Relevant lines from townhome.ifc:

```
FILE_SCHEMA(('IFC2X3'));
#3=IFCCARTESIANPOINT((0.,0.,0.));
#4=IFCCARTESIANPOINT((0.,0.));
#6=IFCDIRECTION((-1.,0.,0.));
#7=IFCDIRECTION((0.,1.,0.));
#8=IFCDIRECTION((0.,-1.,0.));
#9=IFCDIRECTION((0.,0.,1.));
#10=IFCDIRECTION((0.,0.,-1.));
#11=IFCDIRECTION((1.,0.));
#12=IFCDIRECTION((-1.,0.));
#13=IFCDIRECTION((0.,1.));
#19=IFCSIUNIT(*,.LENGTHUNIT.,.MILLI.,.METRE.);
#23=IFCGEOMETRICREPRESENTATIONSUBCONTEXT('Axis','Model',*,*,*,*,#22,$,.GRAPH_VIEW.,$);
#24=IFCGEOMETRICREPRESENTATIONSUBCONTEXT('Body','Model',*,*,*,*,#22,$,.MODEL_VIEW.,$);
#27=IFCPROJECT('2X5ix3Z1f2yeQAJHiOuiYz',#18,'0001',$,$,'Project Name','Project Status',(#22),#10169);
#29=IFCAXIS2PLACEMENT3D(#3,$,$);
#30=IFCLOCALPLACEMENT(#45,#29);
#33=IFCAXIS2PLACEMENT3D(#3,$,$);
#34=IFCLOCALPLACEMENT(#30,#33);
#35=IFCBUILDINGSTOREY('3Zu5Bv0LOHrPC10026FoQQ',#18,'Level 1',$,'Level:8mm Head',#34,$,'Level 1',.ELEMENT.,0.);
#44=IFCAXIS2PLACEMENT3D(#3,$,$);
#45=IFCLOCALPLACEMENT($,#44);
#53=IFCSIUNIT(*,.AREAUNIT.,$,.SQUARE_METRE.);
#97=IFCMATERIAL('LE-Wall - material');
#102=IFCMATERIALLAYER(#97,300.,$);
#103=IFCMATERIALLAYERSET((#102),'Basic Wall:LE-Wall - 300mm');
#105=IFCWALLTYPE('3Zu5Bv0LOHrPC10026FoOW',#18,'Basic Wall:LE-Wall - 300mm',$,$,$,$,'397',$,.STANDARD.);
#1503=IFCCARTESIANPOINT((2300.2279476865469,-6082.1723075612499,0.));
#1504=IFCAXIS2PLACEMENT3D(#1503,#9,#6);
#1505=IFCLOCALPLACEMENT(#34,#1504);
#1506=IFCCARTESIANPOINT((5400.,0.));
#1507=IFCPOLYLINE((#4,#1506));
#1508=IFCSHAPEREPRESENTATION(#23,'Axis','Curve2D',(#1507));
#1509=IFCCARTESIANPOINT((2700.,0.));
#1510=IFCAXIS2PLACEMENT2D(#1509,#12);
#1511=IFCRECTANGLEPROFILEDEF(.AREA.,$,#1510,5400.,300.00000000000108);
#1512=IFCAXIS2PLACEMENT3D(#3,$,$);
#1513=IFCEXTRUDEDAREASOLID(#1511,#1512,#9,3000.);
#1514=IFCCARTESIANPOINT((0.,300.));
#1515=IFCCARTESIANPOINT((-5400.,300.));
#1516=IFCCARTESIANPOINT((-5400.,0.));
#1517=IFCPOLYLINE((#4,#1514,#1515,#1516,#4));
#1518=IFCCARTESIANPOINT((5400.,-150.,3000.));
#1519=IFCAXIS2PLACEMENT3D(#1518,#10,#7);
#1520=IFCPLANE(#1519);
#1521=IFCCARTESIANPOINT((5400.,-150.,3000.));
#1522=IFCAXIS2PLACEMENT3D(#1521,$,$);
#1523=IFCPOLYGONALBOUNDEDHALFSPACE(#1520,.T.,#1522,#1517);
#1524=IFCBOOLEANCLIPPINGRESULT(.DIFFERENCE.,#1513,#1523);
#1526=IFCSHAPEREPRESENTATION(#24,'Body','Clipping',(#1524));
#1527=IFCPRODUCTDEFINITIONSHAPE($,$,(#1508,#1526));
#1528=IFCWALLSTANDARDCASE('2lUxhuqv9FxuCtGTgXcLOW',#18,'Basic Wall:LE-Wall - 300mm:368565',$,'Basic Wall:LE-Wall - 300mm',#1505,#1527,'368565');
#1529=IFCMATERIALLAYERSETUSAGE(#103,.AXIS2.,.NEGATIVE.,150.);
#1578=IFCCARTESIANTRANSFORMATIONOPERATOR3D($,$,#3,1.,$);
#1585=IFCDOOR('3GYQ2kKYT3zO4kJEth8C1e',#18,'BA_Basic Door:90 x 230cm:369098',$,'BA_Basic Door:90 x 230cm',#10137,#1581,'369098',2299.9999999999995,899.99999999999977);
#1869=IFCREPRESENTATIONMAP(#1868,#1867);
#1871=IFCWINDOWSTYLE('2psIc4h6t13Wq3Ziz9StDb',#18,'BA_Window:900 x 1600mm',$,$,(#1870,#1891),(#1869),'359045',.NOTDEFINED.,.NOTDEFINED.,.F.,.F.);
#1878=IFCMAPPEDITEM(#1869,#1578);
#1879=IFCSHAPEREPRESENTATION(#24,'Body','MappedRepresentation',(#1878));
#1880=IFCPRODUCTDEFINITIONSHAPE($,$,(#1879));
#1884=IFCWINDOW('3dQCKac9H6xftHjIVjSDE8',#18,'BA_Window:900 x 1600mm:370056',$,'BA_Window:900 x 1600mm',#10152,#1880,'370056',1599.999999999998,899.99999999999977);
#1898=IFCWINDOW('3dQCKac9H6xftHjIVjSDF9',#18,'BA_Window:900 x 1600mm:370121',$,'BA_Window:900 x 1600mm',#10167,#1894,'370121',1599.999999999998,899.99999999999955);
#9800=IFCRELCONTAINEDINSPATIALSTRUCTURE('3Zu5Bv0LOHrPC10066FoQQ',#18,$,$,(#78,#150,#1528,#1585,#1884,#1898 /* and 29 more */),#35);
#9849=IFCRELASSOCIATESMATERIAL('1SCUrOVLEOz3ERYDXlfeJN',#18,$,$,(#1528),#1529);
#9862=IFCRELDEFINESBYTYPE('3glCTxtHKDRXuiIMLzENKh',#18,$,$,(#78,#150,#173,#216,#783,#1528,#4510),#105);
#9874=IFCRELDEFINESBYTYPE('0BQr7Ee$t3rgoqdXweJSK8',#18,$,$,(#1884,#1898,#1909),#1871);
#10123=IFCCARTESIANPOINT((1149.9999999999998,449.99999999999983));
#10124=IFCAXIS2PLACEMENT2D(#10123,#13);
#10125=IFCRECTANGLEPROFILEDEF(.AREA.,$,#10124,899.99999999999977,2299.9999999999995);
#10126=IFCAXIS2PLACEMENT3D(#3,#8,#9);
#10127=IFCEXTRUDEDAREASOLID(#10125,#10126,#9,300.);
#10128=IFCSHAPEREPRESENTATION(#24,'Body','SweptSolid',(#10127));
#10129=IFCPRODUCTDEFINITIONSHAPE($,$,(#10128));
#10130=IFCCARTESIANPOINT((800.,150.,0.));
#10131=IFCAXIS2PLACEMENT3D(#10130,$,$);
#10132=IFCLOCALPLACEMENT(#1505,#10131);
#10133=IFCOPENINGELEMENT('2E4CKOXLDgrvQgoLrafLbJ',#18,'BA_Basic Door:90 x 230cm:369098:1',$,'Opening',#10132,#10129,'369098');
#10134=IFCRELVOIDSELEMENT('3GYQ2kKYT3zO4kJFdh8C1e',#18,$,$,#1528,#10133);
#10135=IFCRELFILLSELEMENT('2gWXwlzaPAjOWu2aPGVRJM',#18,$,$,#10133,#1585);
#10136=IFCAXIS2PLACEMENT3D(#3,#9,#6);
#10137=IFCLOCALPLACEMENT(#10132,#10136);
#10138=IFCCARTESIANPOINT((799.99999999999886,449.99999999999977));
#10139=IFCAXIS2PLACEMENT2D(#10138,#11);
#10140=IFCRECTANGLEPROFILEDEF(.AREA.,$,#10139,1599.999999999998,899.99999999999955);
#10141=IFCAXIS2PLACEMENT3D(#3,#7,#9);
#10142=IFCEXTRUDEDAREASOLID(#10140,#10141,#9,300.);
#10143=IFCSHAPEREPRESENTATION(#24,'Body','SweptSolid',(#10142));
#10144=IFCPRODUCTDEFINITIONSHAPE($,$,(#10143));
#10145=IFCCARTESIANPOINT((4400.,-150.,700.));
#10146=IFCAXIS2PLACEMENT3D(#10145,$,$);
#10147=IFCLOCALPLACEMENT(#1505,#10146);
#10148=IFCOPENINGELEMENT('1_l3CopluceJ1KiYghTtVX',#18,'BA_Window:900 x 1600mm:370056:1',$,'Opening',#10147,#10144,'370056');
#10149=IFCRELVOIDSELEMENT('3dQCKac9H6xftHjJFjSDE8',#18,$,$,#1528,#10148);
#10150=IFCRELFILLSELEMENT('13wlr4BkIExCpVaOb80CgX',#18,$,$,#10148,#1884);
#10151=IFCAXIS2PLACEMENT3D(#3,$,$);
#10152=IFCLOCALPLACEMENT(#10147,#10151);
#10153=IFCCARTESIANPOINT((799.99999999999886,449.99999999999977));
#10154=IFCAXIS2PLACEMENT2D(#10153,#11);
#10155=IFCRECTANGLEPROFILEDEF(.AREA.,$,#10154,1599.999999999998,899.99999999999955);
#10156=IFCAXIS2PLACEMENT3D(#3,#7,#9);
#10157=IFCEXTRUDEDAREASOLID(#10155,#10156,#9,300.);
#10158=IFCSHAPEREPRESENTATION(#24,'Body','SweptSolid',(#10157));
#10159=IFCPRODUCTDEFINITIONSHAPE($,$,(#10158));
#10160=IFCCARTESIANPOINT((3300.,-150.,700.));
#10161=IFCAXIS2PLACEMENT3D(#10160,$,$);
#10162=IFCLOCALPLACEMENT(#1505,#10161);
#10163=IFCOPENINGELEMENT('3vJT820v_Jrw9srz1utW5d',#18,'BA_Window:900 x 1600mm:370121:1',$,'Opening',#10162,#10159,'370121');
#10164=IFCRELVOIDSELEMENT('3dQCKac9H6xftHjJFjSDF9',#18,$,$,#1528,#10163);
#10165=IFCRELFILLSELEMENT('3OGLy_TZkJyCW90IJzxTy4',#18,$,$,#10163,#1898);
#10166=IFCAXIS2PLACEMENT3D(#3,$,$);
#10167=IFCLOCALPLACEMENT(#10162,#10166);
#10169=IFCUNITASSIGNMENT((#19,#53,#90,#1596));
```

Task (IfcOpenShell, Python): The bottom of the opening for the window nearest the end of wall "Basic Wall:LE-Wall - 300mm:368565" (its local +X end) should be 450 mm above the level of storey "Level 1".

```python
import numpy as np
import ifcopenshell
import ifcopenshell.api.geometry
import ifcopenshell.geom
import ifcopenshell.util.element
import ifcopenshell.util.placement
import ifcopenshell.util.shape
import ifcopenshell.util.unit

model = ifcopenshell.open("townhome.ifc")
unit_scale = ifcopenshell.util.unit.calculate_unit_scale(model)

window = model.by_id(1884)
opening = window.FillsVoids[0].RelatingOpeningElement
storey = ifcopenshell.util.element.get_container(window, ifc_class="IfcBuildingStorey")
level = ifcopenshell.util.placement.get_local_placement(storey.ObjectPlacement)[2, 3]

# The opening's origin need not be at the sill, so measure its lowest point.
shape = ifcopenshell.geom.create_shape(ifcopenshell.geom.settings(), opening)
bottom = ifcopenshell.util.shape.get_shape_bottom_elevation(shape, shape.geometry) / unit_scale
dz = level + 0.45 / unit_scale - bottom

shift = np.array([0.0, 0.0, dz])
# The window is placed relative to its opening, so it follows when the opening moves.
matrix = ifcopenshell.util.placement.get_local_placement(opening.ObjectPlacement)
matrix[:3, 3] += shift
ifcopenshell.api.geometry.edit_object_placement(
    model, product=opening, matrix=matrix, is_si=False, should_transform_children=True
)

print(f"moved by {dz * unit_scale:+.3f} m")

model.write("townhome-out.ifc")
```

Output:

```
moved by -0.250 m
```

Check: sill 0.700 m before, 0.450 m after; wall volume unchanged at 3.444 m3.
